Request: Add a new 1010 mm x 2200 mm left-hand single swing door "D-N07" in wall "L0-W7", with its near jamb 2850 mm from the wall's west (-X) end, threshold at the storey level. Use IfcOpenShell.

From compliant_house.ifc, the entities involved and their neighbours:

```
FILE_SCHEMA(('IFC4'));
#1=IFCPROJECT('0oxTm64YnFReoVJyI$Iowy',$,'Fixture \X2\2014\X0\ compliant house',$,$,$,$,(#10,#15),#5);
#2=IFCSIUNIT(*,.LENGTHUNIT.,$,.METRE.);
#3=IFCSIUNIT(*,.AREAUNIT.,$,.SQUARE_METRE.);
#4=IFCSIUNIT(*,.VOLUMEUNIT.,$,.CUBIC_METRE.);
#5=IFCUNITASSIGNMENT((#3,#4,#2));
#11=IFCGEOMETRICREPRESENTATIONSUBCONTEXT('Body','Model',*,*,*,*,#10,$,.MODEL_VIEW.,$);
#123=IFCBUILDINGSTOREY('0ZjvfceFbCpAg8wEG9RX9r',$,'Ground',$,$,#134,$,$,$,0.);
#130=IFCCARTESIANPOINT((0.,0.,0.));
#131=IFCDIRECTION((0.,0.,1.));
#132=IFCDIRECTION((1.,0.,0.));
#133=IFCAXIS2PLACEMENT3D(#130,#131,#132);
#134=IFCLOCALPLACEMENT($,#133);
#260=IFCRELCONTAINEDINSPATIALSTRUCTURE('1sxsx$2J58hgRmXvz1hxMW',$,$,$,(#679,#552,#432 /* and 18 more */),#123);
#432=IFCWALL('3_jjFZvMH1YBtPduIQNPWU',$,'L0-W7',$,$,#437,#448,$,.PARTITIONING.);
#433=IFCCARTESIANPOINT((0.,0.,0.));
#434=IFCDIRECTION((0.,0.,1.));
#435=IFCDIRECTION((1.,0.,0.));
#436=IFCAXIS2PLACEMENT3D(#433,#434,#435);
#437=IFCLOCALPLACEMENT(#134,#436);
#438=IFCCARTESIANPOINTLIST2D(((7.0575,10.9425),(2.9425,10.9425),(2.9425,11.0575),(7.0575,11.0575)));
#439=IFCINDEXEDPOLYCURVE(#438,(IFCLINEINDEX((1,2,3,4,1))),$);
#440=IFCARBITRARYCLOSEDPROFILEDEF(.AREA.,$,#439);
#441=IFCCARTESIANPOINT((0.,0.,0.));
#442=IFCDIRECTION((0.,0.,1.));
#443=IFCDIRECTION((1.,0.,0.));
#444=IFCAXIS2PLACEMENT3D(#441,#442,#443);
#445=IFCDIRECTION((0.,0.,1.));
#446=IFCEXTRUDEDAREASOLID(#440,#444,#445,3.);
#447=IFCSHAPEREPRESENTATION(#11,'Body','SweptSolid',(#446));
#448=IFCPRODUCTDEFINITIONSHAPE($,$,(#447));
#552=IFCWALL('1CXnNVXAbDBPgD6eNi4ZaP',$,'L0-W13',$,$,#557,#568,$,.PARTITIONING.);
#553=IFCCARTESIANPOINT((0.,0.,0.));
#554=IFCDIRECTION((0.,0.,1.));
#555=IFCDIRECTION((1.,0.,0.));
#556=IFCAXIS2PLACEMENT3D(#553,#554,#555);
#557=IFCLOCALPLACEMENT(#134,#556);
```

```python
import numpy as np
import ifcopenshell
import ifcopenshell.api.feature
import ifcopenshell.api.geometry
import ifcopenshell.api.root
import ifcopenshell.api.spatial
import ifcopenshell.geom
import ifcopenshell.util.element
import ifcopenshell.util.placement
import ifcopenshell.util.representation
import ifcopenshell.util.shape
import ifcopenshell.util.unit

model = ifcopenshell.open("compliant_house.ifc")
unit_scale = ifcopenshell.util.unit.calculate_unit_scale(model)
settings = ifcopenshell.geom.settings()


def volume(element):
    """Net volume in cubic metres, openings subtracted."""
    shape = ifcopenshell.geom.create_shape(settings, element)
    return ifcopenshell.util.shape.get_volume(shape.geometry)


wall = model.by_id(432)
storey = ifcopenshell.util.element.get_container(wall, ifc_class="IfcBuildingStorey")
context = ifcopenshell.util.representation.get_context(model, "Model", "Body", "MODEL_VIEW")
before = volume(wall)

width, height, from_end, sill = 1.01, 2.2, 2.85, 0.0  # metres

# The wall runs along its own X axis, and the end named is its -X end.
wall_shape = ifcopenshell.geom.create_shape(settings, wall)
x, y, z = ifcopenshell.util.shape.get_vertices(wall_shape.geometry).T
start = x.min() + from_end
face, thickness = float(y.min()), float(y.max() - y.min())
wall_matrix = ifcopenshell.util.placement.get_local_placement(wall.ObjectPlacement)
level = ifcopenshell.util.placement.get_local_placement(storey.ObjectPlacement)[2, 3]


def in_wall(x, y):
    """Placement at x, y metres in the wall's axes, at sill height."""
    matrix = wall_matrix.copy()
    matrix[:, 3] = wall_matrix @ np.array([x / unit_scale, y / unit_scale, 0.0, 1.0])
    matrix[2, 3] = level + sill / unit_scale
    return matrix


# Opening: a box that overshoots both wall faces by 50 mm.
opening = ifcopenshell.api.root.create_entity(model, ifc_class="IfcOpeningElement", predefined_type="OPENING")
box = ifcopenshell.api.geometry.add_wall_representation(
    model, context=context, length=width, height=height, thickness=thickness + 0.1
)
ifcopenshell.api.geometry.assign_representation(model, product=opening, representation=box)
ifcopenshell.api.geometry.edit_object_placement(model, product=opening, matrix=in_wall(start, face - 0.05), is_si=False)
ifcopenshell.api.feature.add_feature(model, feature=opening, element=wall)

door = ifcopenshell.api.root.create_entity(model, ifc_class="IfcDoor", name="D-N07", predefined_type="DOOR")
door.OverallWidth, door.OverallHeight = width / unit_scale, height / unit_scale
door.OperationType = "SINGLE_SWING_LEFT"
body = ifcopenshell.api.geometry.add_door_representation(
    model,
    context=context,
    overall_width=door.OverallWidth,
    overall_height=door.OverallHeight,
    operation_type="SINGLE_SWING_LEFT",
    lining_properties={"LiningDepth": thickness / unit_scale, "ThresholdDepth": thickness / unit_scale},
)
ifcopenshell.api.geometry.assign_representation(model, product=door, representation=body)
ifcopenshell.api.spatial.assign_container(model, products=[door], relating_structure=storey)
ifcopenshell.api.feature.add_filling(model, opening=opening, element=door)

# The lining spans the wall, so the door starts at the wall face.
ifcopenshell.api.geometry.edit_object_placement(model, product=door, matrix=in_wall(start, face), is_si=False)

after = volume(wall)

print(f"wall volume {before:.3f} -> {after:.3f} m3")

model.write("compliant_house_rev.ifc")
```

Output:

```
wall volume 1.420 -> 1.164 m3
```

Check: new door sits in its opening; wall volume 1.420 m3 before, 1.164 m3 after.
